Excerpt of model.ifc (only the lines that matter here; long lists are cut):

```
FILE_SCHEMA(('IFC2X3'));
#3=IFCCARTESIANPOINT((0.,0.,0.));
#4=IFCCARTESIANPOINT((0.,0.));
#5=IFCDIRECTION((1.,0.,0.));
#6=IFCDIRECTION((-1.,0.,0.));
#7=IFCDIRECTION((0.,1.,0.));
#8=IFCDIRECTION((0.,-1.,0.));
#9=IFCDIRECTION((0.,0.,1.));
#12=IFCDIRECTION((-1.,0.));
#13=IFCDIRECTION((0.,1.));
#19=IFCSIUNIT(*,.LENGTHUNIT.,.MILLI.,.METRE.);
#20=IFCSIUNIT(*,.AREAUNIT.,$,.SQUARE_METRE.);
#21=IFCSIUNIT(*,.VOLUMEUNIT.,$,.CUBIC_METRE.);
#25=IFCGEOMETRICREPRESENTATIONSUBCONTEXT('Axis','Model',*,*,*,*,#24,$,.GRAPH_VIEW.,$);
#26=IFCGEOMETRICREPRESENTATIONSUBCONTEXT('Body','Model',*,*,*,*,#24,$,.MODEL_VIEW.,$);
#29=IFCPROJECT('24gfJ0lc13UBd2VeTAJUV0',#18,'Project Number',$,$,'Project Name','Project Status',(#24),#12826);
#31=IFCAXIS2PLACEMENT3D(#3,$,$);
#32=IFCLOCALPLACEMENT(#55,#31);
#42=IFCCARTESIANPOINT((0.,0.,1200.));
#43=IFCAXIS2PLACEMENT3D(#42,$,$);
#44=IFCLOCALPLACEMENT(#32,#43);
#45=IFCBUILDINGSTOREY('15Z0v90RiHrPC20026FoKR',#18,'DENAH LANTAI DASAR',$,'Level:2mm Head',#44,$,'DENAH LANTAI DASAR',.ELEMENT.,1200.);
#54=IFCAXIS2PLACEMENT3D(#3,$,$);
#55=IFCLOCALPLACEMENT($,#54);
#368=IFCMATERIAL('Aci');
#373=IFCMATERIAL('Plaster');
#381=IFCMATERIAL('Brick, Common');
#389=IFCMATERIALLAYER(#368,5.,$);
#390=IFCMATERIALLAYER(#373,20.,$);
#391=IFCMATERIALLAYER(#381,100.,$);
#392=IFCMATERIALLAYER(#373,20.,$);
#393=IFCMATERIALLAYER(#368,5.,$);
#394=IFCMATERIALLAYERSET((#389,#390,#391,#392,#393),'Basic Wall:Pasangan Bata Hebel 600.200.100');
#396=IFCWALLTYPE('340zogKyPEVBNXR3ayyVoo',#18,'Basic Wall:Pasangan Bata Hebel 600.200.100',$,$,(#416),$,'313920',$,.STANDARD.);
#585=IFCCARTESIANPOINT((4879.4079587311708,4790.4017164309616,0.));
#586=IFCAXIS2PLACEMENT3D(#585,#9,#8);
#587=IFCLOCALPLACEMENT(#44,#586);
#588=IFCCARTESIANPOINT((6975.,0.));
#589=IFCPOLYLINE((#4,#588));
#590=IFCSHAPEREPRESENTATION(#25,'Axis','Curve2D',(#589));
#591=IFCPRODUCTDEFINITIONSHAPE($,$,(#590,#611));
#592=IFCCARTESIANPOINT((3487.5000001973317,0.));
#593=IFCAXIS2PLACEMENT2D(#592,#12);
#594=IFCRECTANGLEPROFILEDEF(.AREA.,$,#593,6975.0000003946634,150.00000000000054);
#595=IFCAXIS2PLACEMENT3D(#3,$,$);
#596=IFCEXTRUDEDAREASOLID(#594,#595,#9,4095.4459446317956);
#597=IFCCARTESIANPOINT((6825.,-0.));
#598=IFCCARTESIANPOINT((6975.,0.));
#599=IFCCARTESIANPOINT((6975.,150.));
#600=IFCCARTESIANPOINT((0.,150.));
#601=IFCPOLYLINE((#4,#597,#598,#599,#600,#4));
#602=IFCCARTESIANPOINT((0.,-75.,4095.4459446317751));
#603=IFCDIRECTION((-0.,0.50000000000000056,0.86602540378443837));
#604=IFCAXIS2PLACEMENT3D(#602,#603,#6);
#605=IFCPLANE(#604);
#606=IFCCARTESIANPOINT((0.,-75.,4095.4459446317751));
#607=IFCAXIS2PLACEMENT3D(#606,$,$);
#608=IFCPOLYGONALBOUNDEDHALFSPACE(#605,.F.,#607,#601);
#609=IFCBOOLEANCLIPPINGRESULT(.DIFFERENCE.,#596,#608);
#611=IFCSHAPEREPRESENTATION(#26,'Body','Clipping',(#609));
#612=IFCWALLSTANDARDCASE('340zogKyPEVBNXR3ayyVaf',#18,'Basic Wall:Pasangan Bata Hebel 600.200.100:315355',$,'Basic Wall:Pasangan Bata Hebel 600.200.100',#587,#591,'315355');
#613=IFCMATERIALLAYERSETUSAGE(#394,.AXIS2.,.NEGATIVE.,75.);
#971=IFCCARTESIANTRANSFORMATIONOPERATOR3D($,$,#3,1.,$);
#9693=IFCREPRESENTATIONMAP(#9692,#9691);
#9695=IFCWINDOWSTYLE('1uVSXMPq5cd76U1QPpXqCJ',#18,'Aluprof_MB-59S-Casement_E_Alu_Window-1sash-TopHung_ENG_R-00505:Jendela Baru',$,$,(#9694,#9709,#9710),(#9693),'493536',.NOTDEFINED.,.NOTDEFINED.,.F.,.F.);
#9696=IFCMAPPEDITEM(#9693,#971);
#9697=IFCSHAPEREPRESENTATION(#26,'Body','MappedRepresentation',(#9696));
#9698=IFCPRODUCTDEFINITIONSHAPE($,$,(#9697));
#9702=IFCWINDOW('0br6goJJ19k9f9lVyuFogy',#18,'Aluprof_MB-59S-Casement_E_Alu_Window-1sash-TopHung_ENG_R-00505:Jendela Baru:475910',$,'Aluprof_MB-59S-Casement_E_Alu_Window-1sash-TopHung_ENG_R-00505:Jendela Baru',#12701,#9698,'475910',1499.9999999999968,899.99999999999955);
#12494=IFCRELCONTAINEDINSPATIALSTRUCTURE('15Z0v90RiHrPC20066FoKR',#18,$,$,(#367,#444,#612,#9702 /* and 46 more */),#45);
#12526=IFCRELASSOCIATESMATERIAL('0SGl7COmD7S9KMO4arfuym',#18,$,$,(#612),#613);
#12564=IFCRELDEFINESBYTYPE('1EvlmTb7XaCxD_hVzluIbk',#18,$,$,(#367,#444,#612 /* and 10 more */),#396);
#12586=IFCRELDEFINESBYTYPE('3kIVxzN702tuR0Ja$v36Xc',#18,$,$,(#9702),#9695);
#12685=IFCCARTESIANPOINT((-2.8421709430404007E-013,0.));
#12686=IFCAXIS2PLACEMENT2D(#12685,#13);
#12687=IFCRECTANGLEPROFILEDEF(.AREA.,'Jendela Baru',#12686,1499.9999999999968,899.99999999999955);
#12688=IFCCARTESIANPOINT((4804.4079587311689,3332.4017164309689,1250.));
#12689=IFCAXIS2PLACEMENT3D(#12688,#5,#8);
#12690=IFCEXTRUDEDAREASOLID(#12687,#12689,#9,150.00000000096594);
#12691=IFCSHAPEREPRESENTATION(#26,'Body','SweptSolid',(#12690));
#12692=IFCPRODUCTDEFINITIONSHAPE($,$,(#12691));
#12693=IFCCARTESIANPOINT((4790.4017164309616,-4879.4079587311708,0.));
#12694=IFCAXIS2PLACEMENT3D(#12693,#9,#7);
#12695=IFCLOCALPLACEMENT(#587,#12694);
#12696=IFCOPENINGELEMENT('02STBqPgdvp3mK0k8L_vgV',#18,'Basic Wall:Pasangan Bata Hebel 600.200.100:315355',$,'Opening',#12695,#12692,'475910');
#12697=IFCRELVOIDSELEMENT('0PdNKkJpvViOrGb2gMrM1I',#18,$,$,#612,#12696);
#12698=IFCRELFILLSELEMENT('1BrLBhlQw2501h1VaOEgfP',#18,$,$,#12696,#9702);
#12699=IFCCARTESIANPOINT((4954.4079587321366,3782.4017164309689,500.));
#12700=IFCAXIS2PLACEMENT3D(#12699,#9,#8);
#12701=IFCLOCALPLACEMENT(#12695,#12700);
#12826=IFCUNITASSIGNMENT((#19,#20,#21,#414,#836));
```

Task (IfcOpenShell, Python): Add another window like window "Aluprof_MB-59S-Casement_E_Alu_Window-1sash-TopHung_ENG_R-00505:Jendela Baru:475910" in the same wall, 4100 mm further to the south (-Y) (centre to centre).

```python
import ifcopenshell
import ifcopenshell.api.feature
import ifcopenshell.api.geometry
import ifcopenshell.api.root
import ifcopenshell.geom
import ifcopenshell.util.element
import ifcopenshell.util.placement
import ifcopenshell.util.shape
import ifcopenshell.util.unit

model = ifcopenshell.open("model.ifc")
unit_scale = ifcopenshell.util.unit.calculate_unit_scale(model)
settings = ifcopenshell.geom.settings()


def volume(element):
    """Net volume in cubic metres, openings subtracted."""
    shape = ifcopenshell.geom.create_shape(settings, element)
    return ifcopenshell.util.shape.get_volume(shape.geometry)


def reuse_history(source, copy):
    """copy_class also copies each property set's owner history, people and application; keep the originals."""
    for rel in copy.IsDefinedBy:
        if rel.is_a("IfcRelDefinesByProperties") and (history := rel.RelatingPropertyDefinition.OwnerHistory):
            rel.RelatingPropertyDefinition.OwnerHistory = source.OwnerHistory
            ifcopenshell.util.element.remove_deep2(model, history)


window = model.by_guid("0br6goJJ19k9f9lVyuFogy")
opening = window.FillsVoids[0].RelatingOpeningElement
wall = opening.VoidsElements[0].RelatingBuildingElement
before = volume(wall)
shift = ifcopenshell.util.placement.get_local_placement(wall.ObjectPlacement)[:3, 0] * 4.1 / unit_scale

# copy_class copies the void relationship, type, container and properties, but no geometry.
new_opening = ifcopenshell.api.root.copy_class(model, product=opening)
new_opening.Representation = ifcopenshell.util.element.copy_deep(
    model, opening.Representation, exclude=["IfcGeometricRepresentationContext", "IfcRepresentationMap"]
)
new_opening.Name = "Basic Wall:Pasangan Bata Hebel 600.200.100"
new_opening.Tag = None
new_window = ifcopenshell.api.root.copy_class(model, product=window)
new_window.Representation = ifcopenshell.util.element.copy_deep(
    model, window.Representation, exclude=["IfcGeometricRepresentationContext", "IfcRepresentationMap"]
)
new_window.Name = "Aluprof_MB-59S-Casement_E_Alu_Window-1sash-TopHung_ENG_R-00505:Jendela Baru"
new_window.Tag = None
reuse_history(window, new_window)
fills = ifcopenshell.api.feature.add_filling(model, opening=new_opening, element=new_window)
fills.OwnerHistory = new_window.OwnerHistory  # required in IFC2X3

for old, new in ((opening, new_opening), (window, new_window)):
    matrix = ifcopenshell.util.placement.get_local_placement(old.ObjectPlacement)
    matrix[:3, 3] += shift
    ifcopenshell.api.geometry.edit_object_placement(model, product=new, matrix=matrix, is_si=False)

after = volume(wall)

print(f"wall volume {before:.3f} -> {after:.3f} m3")

model.write("model_edited.ifc")
```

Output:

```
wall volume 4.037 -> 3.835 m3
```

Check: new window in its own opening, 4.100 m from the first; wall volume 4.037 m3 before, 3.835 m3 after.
